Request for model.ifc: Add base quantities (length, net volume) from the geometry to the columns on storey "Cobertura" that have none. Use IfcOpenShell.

First a look at what the model holds.

```python
import ifcopenshell
import ifcopenshell.util.element
import ifcopenshell.util.unit

model = ifcopenshell.open("model.ifc")
print(model.schema)
for unit_type in ("LENGTHUNIT", "AREAUNIT", "VOLUMEUNIT"):
    print(unit_type, ifcopenshell.util.unit.calculate_unit_scale(model, unit_type))
storey = next(s for s in model.by_type("IfcBuildingStorey") if s.Name == "Cobertura")
columns = [e for e in ifcopenshell.util.element.get_decomposition(storey) if e.is_a("IfcColumn")]
for e in sorted(columns, key=lambda e: e.id()):
    print(e.id(), e.is_a(), e.Name, list(ifcopenshell.util.element.get_psets(e, qtos_only=True)), sep=" | ")
```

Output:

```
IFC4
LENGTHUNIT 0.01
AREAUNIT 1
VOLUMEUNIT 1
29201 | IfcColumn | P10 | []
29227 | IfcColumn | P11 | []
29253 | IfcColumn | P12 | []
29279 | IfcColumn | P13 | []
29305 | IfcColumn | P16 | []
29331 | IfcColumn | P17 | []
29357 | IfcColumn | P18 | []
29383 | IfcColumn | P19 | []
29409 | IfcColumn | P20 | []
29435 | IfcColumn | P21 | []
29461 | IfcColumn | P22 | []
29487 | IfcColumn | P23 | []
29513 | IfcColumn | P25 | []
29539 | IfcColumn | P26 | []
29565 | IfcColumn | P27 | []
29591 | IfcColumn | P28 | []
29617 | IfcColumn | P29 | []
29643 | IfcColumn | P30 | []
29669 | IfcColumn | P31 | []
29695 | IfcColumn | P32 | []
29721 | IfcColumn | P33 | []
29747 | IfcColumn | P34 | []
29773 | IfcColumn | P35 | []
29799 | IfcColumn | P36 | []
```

```python
import ifcopenshell
import ifcopenshell.api.pset
import ifcopenshell.geom
import ifcopenshell.util.element
import ifcopenshell.util.shape
import ifcopenshell.util.unit

model = ifcopenshell.open("model.ifc")
unit_scale = ifcopenshell.util.unit.calculate_unit_scale(model)
volume_scale = ifcopenshell.util.unit.calculate_unit_scale(model, "VOLUMEUNIT")
settings = ifcopenshell.geom.settings()

storey = next(s for s in model.by_type("IfcBuildingStorey") if s.Name == "Cobertura")
columns = [e for e in ifcopenshell.util.element.get_decomposition(storey) if e.is_a("IfcColumn")]

for e in sorted(columns, key=lambda e: e.id()):
    if ifcopenshell.util.element.get_psets(e, qtos_only=True, should_inherit=False):
        continue
    # Geometry comes back in metres, in the element's own axes.
    shape = ifcopenshell.geom.create_shape(settings, e)
    values = {
        "Length": ifcopenshell.util.shape.get_z(shape.geometry) / unit_scale,
        "NetVolume": ifcopenshell.util.shape.get_volume(shape.geometry) / volume_scale,
    }
    qto = ifcopenshell.api.pset.add_qto(model, product=e, name="Qto_ColumnBaseQuantities")
    ifcopenshell.api.pset.edit_qto(model, qto=qto, properties=values)
    print(e.id(), {k: round(v, 3) for k, v in values.items()})

model.write("model_v2.ifc")
```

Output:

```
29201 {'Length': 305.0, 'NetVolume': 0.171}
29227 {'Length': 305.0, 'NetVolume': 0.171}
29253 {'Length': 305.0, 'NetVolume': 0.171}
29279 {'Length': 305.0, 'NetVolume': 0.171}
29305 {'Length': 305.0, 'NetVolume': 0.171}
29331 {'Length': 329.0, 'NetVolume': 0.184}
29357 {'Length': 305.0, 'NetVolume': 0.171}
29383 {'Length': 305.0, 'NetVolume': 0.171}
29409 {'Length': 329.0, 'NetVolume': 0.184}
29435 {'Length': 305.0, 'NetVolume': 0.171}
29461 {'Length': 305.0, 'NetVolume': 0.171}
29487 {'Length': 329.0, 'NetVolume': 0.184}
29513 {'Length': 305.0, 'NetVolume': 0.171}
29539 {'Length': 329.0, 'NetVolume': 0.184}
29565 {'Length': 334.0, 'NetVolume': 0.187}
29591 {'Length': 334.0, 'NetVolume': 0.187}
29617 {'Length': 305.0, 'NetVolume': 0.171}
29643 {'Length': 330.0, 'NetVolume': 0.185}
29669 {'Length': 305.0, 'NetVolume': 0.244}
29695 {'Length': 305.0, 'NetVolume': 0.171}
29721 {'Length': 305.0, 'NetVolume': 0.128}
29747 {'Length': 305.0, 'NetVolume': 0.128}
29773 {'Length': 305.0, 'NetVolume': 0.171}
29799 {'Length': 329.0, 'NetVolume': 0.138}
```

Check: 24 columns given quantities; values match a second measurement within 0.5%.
